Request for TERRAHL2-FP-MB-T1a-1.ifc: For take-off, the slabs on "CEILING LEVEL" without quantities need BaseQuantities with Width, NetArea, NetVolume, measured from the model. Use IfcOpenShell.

First a look at what the model holds.

```python
import ifcopenshell
import ifcopenshell.util.element
import ifcopenshell.util.unit

model = ifcopenshell.open("TERRAHL2-FP-MB-T1a-1.ifc")
print(model.schema)
for unit_type in ("LENGTHUNIT", "AREAUNIT", "VOLUMEUNIT"):
    print(unit_type, ifcopenshell.util.unit.calculate_unit_scale(model, unit_type))
storey = next(s for s in model.by_type("IfcBuildingStorey") if s.Name == "CEILING LEVEL")
slabs = [e for e in ifcopenshell.util.element.get_decomposition(storey) if e.is_a("IfcSlab")]
for e in sorted(slabs, key=lambda e: e.id()):
    print(e.id(), e.is_a(), e.Name, list(ifcopenshell.util.element.get_psets(e, qtos_only=True)), sep=" | ")
```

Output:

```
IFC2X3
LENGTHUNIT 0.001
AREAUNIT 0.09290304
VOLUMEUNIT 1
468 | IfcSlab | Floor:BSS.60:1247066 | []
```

```python
import ifcopenshell
import ifcopenshell.api.pset
import ifcopenshell.geom
import ifcopenshell.util.element
import ifcopenshell.util.shape
import ifcopenshell.util.unit

model = ifcopenshell.open("TERRAHL2-FP-MB-T1a-1.ifc")
unit_scale = ifcopenshell.util.unit.calculate_unit_scale(model)
area_scale = ifcopenshell.util.unit.calculate_unit_scale(model, "AREAUNIT")
volume_scale = ifcopenshell.util.unit.calculate_unit_scale(model, "VOLUMEUNIT")
settings = ifcopenshell.geom.settings()

storey = next(s for s in model.by_type("IfcBuildingStorey") if s.Name == "CEILING LEVEL")
slabs = [e for e in ifcopenshell.util.element.get_decomposition(storey) if e.is_a("IfcSlab")]

for e in sorted(slabs, key=lambda e: e.id()):
    if ifcopenshell.util.element.get_psets(e, qtos_only=True, should_inherit=False):
        continue
    # Geometry comes back in metres, in the element's own axes.
    shape = ifcopenshell.geom.create_shape(settings, e)
    values = {
        "Width": ifcopenshell.util.shape.get_z(shape.geometry) / unit_scale,
        "NetArea": ifcopenshell.util.shape.get_footprint_area(shape.geometry) / area_scale,
        "NetVolume": ifcopenshell.util.shape.get_volume(shape.geometry) / volume_scale,
    }
    qto = ifcopenshell.api.pset.add_qto(model, product=e, name="BaseQuantities")
    ifcopenshell.api.pset.edit_qto(model, qto=qto, properties=values)
    print(e.id(), {k: round(v, 3) for k, v in values.items()})

model.write("TERRAHL2-FP-MB-T1a-1_updated.ifc")
```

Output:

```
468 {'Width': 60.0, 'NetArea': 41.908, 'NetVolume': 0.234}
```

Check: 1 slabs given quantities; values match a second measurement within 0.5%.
